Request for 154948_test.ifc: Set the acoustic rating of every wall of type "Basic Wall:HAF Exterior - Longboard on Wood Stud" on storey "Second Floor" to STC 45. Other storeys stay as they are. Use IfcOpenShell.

First a look at what the model holds.

```python
import ifcopenshell
import ifcopenshell.util.element

model = ifcopenshell.open("154948_test.ifc")
print(model.schema)
storey = next(s for s in model.by_type("IfcBuildingStorey") if s.Name == "Second Floor")
walls = [e for e in ifcopenshell.util.element.get_decomposition(storey) if e.is_a("IfcWall")]
seen = {}
for e in walls:
    element_type = ifcopenshell.util.element.get_type(e)
    key = (element_type.Name if element_type != e and element_type else None, ifcopenshell.util.element.get_pset(e, "Pset_WallCommon", "AcousticRating"))
    seen[key] = seen.get(key, 0) + 1
for (name, value), count in sorted(seen.items(), key=str):
    print(count, "x", name, "|", value)
```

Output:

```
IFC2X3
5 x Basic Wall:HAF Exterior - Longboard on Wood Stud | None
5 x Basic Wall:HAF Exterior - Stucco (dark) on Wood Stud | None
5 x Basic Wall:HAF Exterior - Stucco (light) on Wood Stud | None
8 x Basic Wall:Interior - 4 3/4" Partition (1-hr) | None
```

```python
import ifcopenshell
import ifcopenshell.api.pset
import ifcopenshell.util.element

model = ifcopenshell.open("154948_test.ifc")

storey = next(s for s in model.by_type("IfcBuildingStorey") if s.Name == "Second Floor")
walls = [e for e in ifcopenshell.util.element.get_decomposition(storey) if e.is_a("IfcWall")]

count = 0
for e in walls:
    element_type = ifcopenshell.util.element.get_type(e)
    if element_type in (None, e) or element_type.Name != "Basic Wall:HAF Exterior - Longboard on Wood Stud":
        continue
    # add_pset returns the element's existing set when there is one.
    pset = ifcopenshell.api.pset.add_pset(model, product=e, name="Pset_WallCommon")
    ifcopenshell.api.pset.edit_pset(model, pset=pset, properties={"AcousticRating": "STC 45"})
    count += 1

print(count, "walls updated")

model.write("154948_test_edited.ifc")
```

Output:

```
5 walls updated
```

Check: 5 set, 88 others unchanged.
